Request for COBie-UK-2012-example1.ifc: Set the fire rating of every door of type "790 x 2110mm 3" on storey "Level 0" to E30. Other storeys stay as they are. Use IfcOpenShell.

First a look at what the model holds.

```python
import ifcopenshell
import ifcopenshell.util.element

model = ifcopenshell.open("COBie-UK-2012-example1.ifc")
print(model.schema)
storey = next(s for s in model.by_type("IfcBuildingStorey") if s.Name == "Level 0")
doors = [e for e in ifcopenshell.util.element.get_decomposition(storey) if e.is_a("IfcDoor")]
seen = {}
for e in doors:
    element_type = ifcopenshell.util.element.get_type(e)
    key = (element_type.Name if element_type != e and element_type else None, ifcopenshell.util.element.get_pset(e, "Pset_DoorCommon", "FireRating"))
    seen[key] = seen.get(key, 0) + 1
for (name, value), count in sorted(seen.items(), key=str):
    print(count, "x", name, "|", value)
```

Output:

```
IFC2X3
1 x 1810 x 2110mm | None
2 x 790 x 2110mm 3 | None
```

```python
import ifcopenshell
import ifcopenshell.api.pset
import ifcopenshell.util.element

model = ifcopenshell.open("COBie-UK-2012-example1.ifc")

storey = next(s for s in model.by_type("IfcBuildingStorey") if s.Name == "Level 0")
doors = [e for e in ifcopenshell.util.element.get_decomposition(storey) if e.is_a("IfcDoor")]

count = 0
for e in doors:
    element_type = ifcopenshell.util.element.get_type(e)
    if element_type in (None, e) or element_type.Name != "790 x 2110mm 3":
        continue
    # add_pset returns the element's existing set when there is one.
    pset = ifcopenshell.api.pset.add_pset(model, product=e, name="Pset_DoorCommon")
    ifcopenshell.api.pset.edit_pset(model, pset=pset, properties={"FireRating": "E30"})
    count += 1

print(count, "doors updated")

model.write("COBie-UK-2012-example1_v2.ifc")
```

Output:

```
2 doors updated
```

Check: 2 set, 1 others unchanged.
